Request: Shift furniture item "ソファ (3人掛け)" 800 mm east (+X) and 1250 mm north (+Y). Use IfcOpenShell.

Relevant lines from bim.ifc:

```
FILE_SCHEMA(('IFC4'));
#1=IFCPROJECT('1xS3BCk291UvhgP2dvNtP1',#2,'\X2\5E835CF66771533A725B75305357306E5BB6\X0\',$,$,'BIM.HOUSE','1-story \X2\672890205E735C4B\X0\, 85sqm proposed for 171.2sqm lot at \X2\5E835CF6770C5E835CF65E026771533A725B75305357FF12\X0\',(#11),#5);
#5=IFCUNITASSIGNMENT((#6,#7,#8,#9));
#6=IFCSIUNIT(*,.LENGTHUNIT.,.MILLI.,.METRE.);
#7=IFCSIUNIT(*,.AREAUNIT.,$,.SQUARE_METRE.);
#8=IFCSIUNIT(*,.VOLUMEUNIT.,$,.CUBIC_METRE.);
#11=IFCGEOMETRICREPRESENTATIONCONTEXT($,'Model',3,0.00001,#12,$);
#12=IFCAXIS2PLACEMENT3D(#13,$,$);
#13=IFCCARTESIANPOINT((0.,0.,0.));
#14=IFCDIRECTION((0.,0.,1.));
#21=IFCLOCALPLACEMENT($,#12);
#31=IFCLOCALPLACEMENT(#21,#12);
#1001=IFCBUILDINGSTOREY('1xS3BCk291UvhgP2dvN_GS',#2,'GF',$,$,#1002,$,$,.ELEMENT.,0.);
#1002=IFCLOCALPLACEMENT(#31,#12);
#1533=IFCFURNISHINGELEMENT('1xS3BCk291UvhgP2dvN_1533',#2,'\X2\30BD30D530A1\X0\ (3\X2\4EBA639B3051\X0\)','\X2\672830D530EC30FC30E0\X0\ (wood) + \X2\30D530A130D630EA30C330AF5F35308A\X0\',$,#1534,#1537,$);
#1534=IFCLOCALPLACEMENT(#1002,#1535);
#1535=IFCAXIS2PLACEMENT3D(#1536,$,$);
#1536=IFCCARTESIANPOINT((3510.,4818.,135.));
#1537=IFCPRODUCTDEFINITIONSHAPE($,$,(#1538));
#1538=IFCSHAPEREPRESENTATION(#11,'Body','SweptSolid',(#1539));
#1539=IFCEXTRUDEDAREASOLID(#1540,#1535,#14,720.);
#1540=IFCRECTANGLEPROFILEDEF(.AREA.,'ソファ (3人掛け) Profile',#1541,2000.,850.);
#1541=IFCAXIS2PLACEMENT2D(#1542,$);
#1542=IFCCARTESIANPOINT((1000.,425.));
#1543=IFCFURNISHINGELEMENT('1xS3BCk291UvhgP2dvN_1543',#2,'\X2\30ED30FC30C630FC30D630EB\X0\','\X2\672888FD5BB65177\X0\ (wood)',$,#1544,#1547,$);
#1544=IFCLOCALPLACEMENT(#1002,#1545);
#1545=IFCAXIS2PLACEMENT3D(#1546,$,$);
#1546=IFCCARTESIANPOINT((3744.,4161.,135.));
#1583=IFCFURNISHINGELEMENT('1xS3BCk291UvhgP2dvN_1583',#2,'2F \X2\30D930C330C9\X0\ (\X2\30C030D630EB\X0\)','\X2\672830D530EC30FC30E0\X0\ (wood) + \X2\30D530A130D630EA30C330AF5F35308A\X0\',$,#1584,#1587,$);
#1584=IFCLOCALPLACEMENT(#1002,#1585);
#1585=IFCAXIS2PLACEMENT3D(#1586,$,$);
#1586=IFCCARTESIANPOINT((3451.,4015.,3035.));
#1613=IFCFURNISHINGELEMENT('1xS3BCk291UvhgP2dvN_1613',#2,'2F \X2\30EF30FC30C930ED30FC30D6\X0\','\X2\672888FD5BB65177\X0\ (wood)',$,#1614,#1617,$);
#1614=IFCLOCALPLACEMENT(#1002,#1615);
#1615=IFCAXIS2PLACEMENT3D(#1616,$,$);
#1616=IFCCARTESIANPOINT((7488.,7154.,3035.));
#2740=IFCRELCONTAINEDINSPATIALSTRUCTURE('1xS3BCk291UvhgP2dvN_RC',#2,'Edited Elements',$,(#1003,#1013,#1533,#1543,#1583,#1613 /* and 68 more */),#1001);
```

```python
import ifcopenshell
import ifcopenshell.api.geometry
import ifcopenshell.util.placement

model = ifcopenshell.open("bim.ifc")

item = model.by_guid("1xS3BCk291UvhgP2dvN_1533")
matrix = ifcopenshell.util.placement.get_local_placement(item.ObjectPlacement)
matrix[0, 3] += 800.0
matrix[1, 3] += 1250.0
ifcopenshell.api.geometry.edit_object_placement(model, product=item, matrix=matrix, is_si=False)

print(ifcopenshell.util.placement.get_local_placement(item.ObjectPlacement).round(3) + 0.0)

model.write("bim_updated.ifc")
```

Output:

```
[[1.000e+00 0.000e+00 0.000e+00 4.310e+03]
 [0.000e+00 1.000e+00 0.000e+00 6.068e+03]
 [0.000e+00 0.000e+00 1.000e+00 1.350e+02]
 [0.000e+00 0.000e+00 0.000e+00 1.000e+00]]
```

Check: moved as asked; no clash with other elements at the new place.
